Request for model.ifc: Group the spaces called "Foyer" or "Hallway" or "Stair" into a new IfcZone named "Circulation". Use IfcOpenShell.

First a look at what the model holds.

```python
import ifcopenshell

model = ifcopenshell.open("model.ifc")
print(model.schema)
seen = {}
for space in model.by_type("IfcSpace"):
    seen[space.LongName] = seen.get(space.LongName, 0) + 1
for name, count in sorted(seen.items(), key=str):
    print(count, "x", name)
print("zones:", [z.Name for z in model.by_type("IfcZone")][:20])
```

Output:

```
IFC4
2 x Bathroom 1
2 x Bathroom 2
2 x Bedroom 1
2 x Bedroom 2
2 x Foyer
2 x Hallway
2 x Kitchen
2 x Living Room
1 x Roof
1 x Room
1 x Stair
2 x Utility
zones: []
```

```python
import ifcopenshell
import ifcopenshell.api.group
import ifcopenshell.api.root

model = ifcopenshell.open("model.ifc")

names = {"Foyer", "Hallway", "Stair"}
spaces = [s for s in model.by_type("IfcSpace") if s.LongName in names]

zone = ifcopenshell.api.root.create_entity(model, ifc_class="IfcZone", name="Circulation")
ifcopenshell.api.group.assign_group(model, products=spaces, group=zone)
print(len(spaces), "spaces in", zone.Name)

model.write("model_v2.ifc")
```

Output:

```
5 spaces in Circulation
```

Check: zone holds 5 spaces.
